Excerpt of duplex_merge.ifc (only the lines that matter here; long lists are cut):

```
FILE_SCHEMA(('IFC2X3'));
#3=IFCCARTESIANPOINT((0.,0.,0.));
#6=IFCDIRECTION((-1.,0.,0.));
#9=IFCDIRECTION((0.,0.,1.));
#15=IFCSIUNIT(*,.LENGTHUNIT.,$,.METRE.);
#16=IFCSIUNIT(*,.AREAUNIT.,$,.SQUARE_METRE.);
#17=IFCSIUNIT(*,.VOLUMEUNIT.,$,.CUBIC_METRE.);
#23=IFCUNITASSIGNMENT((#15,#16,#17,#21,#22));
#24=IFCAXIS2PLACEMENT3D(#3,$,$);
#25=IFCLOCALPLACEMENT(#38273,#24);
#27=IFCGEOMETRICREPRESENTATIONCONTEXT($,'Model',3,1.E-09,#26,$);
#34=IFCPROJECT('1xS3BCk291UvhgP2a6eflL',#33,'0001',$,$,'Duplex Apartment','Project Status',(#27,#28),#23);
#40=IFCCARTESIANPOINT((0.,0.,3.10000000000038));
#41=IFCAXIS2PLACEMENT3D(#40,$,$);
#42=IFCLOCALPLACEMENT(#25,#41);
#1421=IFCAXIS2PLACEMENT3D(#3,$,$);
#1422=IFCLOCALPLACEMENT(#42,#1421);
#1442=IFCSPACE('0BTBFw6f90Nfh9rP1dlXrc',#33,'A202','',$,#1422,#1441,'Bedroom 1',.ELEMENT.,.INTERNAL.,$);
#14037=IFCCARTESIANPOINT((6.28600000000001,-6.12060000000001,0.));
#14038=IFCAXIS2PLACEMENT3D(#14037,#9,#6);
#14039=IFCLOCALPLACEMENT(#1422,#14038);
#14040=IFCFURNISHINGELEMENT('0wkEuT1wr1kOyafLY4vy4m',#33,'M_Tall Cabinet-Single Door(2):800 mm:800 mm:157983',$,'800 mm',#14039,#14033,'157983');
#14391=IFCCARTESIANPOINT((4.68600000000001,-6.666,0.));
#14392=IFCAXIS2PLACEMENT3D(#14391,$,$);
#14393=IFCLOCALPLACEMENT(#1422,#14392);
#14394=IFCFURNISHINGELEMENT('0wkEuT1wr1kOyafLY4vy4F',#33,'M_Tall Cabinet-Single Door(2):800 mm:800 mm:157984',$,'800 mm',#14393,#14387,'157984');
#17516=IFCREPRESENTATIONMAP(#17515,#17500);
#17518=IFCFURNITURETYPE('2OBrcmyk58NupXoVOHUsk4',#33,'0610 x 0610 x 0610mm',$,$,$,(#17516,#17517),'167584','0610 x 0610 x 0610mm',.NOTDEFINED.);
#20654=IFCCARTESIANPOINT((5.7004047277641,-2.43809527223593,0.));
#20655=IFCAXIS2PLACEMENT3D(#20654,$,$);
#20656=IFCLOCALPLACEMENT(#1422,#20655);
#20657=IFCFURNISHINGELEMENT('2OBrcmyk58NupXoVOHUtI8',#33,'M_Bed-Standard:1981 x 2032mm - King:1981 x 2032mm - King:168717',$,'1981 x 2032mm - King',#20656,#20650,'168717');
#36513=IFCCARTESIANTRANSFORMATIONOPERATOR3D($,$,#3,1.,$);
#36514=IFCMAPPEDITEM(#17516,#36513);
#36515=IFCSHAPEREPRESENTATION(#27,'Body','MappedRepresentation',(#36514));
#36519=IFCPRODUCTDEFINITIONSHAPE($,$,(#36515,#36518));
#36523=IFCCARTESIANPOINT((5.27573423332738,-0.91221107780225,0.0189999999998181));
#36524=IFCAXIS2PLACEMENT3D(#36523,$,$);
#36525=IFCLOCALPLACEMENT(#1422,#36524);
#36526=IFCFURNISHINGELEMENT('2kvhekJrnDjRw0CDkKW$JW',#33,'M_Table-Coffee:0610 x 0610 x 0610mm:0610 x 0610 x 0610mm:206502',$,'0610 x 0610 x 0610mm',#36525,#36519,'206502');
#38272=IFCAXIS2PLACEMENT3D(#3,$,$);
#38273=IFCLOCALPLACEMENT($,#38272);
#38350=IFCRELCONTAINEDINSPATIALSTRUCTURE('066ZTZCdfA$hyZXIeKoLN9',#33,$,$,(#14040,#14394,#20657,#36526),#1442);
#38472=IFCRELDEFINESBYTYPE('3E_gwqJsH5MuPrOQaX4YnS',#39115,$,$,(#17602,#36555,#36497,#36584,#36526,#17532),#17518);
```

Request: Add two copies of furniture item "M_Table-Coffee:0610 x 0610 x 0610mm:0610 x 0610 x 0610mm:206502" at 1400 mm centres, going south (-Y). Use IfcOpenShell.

```python
import numpy as np
import ifcopenshell
import ifcopenshell.api.geometry
import ifcopenshell.api.root
import ifcopenshell.util.element
import ifcopenshell.util.placement
import ifcopenshell.util.unit

model = ifcopenshell.open("duplex_merge.ifc")
unit_scale = ifcopenshell.util.unit.calculate_unit_scale(model)


def reuse_history(source, copy):
    """copy_class also copies each property set's owner history, people and application; keep the originals."""
    for rel in copy.IsDefinedBy:
        if rel.is_a("IfcRelDefinesByProperties") and (history := rel.RelatingPropertyDefinition.OwnerHistory):
            rel.RelatingPropertyDefinition.OwnerHistory = source.OwnerHistory
            ifcopenshell.util.element.remove_deep2(model, history)


source = model.by_id(36526)
base = ifcopenshell.util.placement.get_local_placement(source.ObjectPlacement)
step = np.array([0.0, -1.0, 0.0]) * 1.4 / unit_scale

for i in range(1, 3):
    copy = ifcopenshell.api.root.copy_class(model, product=source)
    copy.Representation = ifcopenshell.util.element.copy_deep(
        model, source.Representation, exclude=["IfcGeometricRepresentationContext", "IfcRepresentationMap"]
    )
    copy.Name = "M_Table-Coffee:0610 x 0610 x 0610mm:0610 x 0610 x 0610mm"
    copy.Tag = None
    reuse_history(source, copy)
    matrix = base.copy()
    matrix[:3, 3] += i * step
    print("added at", matrix[:3, 3].round(3) + 0.0)
    ifcopenshell.api.geometry.edit_object_placement(model, product=copy, matrix=matrix, is_si=False)

model.write("duplex_merge_edited.ifc")
```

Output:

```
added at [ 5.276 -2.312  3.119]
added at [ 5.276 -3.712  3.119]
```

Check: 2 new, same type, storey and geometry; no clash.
